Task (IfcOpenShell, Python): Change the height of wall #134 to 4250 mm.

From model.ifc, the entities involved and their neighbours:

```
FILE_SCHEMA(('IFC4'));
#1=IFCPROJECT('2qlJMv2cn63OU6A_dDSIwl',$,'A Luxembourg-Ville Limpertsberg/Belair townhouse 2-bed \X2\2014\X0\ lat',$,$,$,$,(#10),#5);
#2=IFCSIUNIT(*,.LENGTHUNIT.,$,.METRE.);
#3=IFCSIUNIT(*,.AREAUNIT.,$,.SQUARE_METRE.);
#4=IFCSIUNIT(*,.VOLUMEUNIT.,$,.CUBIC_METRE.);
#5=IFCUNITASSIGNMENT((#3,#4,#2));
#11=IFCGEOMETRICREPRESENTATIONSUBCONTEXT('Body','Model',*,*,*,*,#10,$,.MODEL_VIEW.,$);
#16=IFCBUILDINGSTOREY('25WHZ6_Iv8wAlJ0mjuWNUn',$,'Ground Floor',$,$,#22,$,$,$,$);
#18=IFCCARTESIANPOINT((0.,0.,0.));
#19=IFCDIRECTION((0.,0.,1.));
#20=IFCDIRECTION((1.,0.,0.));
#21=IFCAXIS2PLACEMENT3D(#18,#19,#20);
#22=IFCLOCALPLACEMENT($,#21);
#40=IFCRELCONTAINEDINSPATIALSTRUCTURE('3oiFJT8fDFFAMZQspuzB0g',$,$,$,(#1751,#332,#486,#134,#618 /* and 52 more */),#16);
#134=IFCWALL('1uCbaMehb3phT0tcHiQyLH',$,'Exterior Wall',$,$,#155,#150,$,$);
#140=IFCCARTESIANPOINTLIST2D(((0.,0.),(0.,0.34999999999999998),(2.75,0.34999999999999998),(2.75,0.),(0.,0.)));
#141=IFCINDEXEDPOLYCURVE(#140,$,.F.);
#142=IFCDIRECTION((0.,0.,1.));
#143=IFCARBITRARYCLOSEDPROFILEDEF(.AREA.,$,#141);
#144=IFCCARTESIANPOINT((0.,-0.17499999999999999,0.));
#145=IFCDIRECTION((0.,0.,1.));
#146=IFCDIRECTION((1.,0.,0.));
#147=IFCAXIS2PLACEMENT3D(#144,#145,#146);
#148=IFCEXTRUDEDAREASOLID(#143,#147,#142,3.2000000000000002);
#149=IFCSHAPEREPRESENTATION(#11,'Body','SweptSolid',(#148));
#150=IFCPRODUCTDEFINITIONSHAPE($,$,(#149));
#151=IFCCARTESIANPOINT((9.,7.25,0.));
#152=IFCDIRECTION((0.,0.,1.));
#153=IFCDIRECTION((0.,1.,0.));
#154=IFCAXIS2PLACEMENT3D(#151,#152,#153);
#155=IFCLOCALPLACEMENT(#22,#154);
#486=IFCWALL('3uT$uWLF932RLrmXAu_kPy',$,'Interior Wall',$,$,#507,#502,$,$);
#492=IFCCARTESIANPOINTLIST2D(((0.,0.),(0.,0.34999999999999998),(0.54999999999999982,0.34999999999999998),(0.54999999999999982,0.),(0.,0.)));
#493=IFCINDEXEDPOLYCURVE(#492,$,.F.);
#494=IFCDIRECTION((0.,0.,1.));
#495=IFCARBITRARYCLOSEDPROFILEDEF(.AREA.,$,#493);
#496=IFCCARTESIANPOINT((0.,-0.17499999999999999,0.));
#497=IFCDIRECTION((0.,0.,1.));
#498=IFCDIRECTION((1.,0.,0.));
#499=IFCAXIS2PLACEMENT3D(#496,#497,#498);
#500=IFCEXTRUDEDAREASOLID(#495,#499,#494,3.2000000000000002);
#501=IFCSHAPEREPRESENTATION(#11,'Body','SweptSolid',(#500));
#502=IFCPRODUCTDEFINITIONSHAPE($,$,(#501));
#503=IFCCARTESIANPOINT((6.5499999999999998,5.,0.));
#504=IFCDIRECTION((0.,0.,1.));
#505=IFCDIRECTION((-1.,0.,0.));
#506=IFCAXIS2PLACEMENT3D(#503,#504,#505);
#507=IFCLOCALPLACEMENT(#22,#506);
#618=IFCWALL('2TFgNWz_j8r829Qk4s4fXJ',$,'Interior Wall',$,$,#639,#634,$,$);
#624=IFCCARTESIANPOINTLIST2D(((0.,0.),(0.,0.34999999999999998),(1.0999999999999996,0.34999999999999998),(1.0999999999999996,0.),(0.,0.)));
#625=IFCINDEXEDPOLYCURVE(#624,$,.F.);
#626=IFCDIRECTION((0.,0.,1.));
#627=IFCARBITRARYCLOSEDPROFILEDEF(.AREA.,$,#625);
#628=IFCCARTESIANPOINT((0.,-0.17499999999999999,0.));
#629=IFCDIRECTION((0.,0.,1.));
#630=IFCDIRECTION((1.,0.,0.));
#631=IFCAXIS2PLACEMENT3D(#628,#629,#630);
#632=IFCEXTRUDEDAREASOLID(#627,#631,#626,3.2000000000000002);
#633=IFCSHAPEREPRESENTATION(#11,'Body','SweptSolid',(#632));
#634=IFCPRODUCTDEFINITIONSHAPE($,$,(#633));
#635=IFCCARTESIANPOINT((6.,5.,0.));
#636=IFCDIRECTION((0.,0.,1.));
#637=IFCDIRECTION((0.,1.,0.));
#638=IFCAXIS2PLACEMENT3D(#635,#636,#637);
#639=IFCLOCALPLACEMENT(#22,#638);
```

```python
import ifcopenshell
import ifcopenshell.geom
import ifcopenshell.util.representation
import ifcopenshell.util.shape
import ifcopenshell.util.unit

model = ifcopenshell.open("model.ifc")
unit_scale = ifcopenshell.util.unit.calculate_unit_scale(model)
settings = ifcopenshell.geom.settings()


def volume(element):
    """Net volume in cubic metres, openings subtracted."""
    shape = ifcopenshell.geom.create_shape(settings, element)
    return ifcopenshell.util.shape.get_volume(shape.geometry)


wall = model.by_id(134)
before = volume(wall)

body = ifcopenshell.util.representation.get_representation(wall, "Model", "Body")
solid = body.Items[0]
old_height = solid.Depth
solid.Depth = 4.25 / unit_scale
after = volume(wall)

print(f"height {old_height:g} -> {solid.Depth:g}, volume {before:.3f} -> {after:.3f} m3")

model.write("model_updated.ifc")
```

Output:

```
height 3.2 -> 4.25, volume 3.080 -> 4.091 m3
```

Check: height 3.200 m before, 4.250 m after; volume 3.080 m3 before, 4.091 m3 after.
